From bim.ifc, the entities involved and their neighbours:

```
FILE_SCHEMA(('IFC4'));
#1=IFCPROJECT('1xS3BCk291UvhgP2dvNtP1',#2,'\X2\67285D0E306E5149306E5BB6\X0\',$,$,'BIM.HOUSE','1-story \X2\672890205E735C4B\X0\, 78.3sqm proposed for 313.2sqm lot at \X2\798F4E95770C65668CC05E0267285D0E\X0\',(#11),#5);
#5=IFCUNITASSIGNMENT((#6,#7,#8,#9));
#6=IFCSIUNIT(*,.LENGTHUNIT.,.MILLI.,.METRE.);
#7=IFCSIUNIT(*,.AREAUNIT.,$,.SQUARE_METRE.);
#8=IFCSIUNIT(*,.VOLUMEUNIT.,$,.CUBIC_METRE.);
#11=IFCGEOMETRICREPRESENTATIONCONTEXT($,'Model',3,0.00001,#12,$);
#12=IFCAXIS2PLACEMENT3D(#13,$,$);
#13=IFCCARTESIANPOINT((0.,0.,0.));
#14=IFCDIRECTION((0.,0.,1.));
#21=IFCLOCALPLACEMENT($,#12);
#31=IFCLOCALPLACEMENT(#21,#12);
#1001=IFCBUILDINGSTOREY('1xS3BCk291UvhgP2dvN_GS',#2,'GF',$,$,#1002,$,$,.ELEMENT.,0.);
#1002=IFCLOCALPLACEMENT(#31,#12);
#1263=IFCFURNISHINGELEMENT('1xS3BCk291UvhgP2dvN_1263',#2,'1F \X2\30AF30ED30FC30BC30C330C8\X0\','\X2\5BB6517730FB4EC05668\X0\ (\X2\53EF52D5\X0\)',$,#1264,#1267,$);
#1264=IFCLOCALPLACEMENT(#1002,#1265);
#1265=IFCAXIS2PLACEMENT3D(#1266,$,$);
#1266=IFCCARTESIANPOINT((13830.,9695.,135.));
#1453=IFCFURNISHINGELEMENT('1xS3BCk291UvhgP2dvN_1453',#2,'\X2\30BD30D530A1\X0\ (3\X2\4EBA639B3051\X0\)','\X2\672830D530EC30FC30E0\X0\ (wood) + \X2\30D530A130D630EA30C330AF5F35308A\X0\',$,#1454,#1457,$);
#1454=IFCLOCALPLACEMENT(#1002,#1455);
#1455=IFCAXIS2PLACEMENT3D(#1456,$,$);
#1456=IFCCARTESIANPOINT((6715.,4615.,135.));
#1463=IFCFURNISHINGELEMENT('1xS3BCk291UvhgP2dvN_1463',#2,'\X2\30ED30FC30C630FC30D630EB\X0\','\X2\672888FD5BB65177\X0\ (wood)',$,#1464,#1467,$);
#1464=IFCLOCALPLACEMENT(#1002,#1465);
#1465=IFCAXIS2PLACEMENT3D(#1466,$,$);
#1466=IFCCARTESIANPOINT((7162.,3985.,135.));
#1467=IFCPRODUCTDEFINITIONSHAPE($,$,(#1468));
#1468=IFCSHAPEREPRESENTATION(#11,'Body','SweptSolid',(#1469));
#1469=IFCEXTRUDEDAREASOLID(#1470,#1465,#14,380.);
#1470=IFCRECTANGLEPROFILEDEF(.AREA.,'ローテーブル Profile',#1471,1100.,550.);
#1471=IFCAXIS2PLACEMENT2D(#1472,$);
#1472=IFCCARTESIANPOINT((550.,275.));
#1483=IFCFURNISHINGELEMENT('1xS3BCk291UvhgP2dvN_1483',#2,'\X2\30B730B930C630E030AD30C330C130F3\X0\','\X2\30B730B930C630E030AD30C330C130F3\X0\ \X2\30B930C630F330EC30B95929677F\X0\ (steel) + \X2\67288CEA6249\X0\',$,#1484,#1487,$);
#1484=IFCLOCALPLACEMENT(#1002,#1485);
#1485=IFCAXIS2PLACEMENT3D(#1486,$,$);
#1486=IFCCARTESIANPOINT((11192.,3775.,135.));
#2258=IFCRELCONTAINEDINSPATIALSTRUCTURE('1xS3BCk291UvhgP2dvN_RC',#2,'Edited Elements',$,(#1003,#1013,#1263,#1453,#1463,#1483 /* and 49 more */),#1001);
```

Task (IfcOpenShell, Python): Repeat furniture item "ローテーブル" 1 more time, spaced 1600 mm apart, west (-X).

```python
import numpy as np
import ifcopenshell
import ifcopenshell.api.geometry
import ifcopenshell.api.root
import ifcopenshell.util.element
import ifcopenshell.util.placement
import ifcopenshell.util.unit

model = ifcopenshell.open("bim.ifc")
unit_scale = ifcopenshell.util.unit.calculate_unit_scale(model)


def reuse_history(source, copy):
    """copy_class also copies each property set's owner history, people and application; keep the originals."""
    for rel in copy.IsDefinedBy:
        if rel.is_a("IfcRelDefinesByProperties") and (history := rel.RelatingPropertyDefinition.OwnerHistory):
            rel.RelatingPropertyDefinition.OwnerHistory = source.OwnerHistory
            ifcopenshell.util.element.remove_deep2(model, history)


source = model.by_id(1463)
base = ifcopenshell.util.placement.get_local_placement(source.ObjectPlacement)
step = np.array([-1.0, 0.0, 0.0]) * 1.6 / unit_scale

for i in range(1, 2):
    copy = ifcopenshell.api.root.copy_class(model, product=source)
    copy.Representation = ifcopenshell.util.element.copy_deep(
        model, source.Representation, exclude=["IfcGeometricRepresentationContext", "IfcRepresentationMap"]
    )
    reuse_history(source, copy)
    matrix = base.copy()
    matrix[:3, 3] += i * step
    print("added at", matrix[:3, 3].round(3) + 0.0)
    ifcopenshell.api.geometry.edit_object_placement(model, product=copy, matrix=matrix, is_si=False)

model.write("bim-out.ifc")
```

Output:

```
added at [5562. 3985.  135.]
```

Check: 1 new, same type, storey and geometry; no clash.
